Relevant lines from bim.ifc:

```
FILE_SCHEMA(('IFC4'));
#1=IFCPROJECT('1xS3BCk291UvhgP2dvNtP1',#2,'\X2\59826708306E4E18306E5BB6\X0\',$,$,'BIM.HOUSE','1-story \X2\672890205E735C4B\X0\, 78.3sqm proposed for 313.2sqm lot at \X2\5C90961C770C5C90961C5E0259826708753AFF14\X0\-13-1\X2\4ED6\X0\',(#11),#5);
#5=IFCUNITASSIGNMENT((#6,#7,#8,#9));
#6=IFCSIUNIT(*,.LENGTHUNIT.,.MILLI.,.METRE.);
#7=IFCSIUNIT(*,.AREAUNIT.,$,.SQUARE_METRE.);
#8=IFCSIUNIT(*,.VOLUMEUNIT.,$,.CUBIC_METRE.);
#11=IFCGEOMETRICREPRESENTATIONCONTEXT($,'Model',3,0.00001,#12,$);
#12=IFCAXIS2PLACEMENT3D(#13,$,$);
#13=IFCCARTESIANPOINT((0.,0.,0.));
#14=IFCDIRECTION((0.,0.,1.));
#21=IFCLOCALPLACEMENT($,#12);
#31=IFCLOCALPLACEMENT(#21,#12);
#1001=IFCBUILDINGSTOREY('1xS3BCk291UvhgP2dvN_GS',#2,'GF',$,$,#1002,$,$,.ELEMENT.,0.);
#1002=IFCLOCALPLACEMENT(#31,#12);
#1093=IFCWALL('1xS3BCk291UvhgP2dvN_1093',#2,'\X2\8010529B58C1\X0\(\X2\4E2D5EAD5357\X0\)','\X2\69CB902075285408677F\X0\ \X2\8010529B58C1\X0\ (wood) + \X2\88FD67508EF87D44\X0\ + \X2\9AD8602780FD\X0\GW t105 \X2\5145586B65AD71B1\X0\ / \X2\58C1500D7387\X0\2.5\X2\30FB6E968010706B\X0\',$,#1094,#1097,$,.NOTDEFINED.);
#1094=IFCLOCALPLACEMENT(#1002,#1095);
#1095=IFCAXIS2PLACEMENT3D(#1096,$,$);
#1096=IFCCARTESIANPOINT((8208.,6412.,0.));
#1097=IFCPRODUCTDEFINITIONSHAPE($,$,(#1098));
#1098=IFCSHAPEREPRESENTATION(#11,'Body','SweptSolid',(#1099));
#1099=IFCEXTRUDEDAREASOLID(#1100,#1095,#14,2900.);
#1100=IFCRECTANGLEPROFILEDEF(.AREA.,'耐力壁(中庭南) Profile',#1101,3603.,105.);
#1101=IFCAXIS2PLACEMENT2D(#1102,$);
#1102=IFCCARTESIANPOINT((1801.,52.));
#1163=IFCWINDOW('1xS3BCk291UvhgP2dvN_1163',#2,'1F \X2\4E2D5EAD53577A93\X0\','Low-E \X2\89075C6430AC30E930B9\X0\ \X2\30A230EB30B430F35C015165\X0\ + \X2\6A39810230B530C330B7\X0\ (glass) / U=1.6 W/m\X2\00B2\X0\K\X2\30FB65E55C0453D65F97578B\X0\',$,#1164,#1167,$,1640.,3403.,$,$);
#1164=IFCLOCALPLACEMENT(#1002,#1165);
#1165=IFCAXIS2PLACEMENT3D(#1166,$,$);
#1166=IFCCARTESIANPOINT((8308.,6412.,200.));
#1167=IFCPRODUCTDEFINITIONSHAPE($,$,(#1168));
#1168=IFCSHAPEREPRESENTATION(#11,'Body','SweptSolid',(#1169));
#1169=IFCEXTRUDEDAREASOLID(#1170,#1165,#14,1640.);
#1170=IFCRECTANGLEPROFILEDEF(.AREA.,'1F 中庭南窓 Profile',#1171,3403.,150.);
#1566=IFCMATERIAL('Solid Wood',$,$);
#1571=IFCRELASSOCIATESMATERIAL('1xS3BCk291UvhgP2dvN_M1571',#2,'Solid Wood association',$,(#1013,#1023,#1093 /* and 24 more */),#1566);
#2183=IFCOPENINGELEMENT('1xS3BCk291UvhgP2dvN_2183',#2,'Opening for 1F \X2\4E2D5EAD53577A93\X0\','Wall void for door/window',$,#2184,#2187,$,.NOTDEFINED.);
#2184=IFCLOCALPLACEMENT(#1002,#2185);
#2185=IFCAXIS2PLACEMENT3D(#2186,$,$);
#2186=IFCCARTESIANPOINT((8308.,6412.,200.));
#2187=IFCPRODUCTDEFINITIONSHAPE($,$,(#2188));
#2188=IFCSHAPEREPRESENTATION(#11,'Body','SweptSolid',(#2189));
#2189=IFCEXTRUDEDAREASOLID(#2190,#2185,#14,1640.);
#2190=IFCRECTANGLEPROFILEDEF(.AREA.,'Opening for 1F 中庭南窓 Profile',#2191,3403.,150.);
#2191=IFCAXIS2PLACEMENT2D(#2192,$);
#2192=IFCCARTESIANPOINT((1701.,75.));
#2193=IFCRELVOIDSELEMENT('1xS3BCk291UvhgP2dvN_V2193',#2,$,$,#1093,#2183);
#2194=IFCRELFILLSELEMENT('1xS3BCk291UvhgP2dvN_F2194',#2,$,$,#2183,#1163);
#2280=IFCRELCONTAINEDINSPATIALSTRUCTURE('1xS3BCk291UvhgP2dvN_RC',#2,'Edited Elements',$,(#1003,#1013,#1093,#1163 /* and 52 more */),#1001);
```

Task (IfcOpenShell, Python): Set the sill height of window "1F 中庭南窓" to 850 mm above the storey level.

```python
import numpy as np
import ifcopenshell
import ifcopenshell.api.geometry
import ifcopenshell.geom
import ifcopenshell.util.element
import ifcopenshell.util.placement
import ifcopenshell.util.shape
import ifcopenshell.util.unit

model = ifcopenshell.open("bim.ifc")
unit_scale = ifcopenshell.util.unit.calculate_unit_scale(model)

window = model.by_guid("1xS3BCk291UvhgP2dvN_1163")
opening = window.FillsVoids[0].RelatingOpeningElement
storey = ifcopenshell.util.element.get_container(window, ifc_class="IfcBuildingStorey")
level = ifcopenshell.util.placement.get_local_placement(storey.ObjectPlacement)[2, 3]

# The opening's origin need not be at the sill, so measure its lowest point.
shape = ifcopenshell.geom.create_shape(ifcopenshell.geom.settings(), opening)
bottom = ifcopenshell.util.shape.get_shape_bottom_elevation(shape, shape.geometry) / unit_scale
dz = level + 0.85 / unit_scale - bottom

shift = np.array([0.0, 0.0, dz])
# The window is not placed relative to its opening, so move both.
for product in (opening, window):
    matrix = ifcopenshell.util.placement.get_local_placement(product.ObjectPlacement)
    matrix[:3, 3] += shift
    ifcopenshell.api.geometry.edit_object_placement(model, product=product, matrix=matrix, is_si=False)

print(f"moved by {dz * unit_scale:+.3f} m")

model.write("bim-out.ifc")
```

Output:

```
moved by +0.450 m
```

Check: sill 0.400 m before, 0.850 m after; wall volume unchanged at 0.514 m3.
